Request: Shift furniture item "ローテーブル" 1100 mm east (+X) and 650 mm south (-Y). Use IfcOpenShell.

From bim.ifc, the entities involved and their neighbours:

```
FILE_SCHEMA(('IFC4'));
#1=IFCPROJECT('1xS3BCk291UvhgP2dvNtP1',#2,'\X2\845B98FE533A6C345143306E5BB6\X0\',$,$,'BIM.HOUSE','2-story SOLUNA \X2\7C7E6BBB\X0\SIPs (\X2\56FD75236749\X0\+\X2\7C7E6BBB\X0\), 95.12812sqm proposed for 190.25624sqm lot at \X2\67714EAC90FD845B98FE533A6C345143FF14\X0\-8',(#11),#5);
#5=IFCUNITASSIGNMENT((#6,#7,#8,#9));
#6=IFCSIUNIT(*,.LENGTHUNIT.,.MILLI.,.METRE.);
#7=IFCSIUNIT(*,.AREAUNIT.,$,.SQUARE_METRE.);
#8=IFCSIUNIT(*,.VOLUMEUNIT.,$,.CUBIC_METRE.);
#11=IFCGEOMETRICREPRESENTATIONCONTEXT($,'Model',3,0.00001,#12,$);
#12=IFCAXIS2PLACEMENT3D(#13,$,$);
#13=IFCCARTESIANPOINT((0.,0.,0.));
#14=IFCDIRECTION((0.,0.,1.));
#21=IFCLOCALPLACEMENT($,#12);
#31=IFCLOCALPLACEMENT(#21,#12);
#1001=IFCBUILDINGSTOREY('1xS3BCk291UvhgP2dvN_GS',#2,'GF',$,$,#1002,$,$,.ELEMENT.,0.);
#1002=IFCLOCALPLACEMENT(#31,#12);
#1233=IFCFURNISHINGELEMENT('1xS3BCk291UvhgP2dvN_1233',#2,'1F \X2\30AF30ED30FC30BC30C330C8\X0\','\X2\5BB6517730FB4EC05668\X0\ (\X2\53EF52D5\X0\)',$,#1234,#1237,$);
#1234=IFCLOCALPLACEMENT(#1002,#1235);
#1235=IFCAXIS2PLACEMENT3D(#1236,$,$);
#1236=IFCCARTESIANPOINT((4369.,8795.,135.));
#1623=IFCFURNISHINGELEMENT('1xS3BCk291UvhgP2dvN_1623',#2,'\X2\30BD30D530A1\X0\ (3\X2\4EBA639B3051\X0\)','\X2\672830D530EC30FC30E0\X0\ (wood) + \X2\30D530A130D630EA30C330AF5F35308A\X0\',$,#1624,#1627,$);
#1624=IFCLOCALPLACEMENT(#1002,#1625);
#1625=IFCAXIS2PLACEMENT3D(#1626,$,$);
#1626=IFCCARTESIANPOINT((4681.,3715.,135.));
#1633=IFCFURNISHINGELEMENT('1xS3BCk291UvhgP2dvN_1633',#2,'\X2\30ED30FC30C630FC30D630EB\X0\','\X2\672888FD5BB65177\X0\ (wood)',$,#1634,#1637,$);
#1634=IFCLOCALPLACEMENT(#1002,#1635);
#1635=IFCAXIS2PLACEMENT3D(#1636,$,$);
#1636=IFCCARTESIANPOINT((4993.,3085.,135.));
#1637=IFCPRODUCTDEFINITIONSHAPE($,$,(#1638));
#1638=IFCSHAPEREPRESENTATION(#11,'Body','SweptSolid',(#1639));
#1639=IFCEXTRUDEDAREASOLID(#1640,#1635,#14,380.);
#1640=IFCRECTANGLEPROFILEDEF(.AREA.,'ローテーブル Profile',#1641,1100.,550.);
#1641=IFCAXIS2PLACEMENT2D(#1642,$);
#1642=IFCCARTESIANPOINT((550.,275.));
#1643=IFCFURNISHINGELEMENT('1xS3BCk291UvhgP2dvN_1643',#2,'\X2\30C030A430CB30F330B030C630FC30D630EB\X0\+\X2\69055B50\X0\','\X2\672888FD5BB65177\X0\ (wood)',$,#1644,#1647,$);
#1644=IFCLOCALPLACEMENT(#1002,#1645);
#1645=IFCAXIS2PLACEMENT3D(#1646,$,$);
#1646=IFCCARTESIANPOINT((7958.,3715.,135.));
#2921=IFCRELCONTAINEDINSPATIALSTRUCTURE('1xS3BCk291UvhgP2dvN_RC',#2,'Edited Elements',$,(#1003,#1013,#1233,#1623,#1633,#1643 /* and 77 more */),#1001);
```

```python
import ifcopenshell
import ifcopenshell.api.geometry
import ifcopenshell.util.placement
import ifcopenshell.util.unit

model = ifcopenshell.open("bim.ifc")
unit_scale = ifcopenshell.util.unit.calculate_unit_scale(model)

item = model.by_guid("1xS3BCk291UvhgP2dvN_1633")
matrix = ifcopenshell.util.placement.get_local_placement(item.ObjectPlacement)
matrix[0, 3] += 1.1 / unit_scale
matrix[1, 3] -= 0.65 / unit_scale
ifcopenshell.api.geometry.edit_object_placement(model, product=item, matrix=matrix, is_si=False)

print(ifcopenshell.util.placement.get_local_placement(item.ObjectPlacement).round(3) + 0.0)

model.write("bim-out.ifc")
```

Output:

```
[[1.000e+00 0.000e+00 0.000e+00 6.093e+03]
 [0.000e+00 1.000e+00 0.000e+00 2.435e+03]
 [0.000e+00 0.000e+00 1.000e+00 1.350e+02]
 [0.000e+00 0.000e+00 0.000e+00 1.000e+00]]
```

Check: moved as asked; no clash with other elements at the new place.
